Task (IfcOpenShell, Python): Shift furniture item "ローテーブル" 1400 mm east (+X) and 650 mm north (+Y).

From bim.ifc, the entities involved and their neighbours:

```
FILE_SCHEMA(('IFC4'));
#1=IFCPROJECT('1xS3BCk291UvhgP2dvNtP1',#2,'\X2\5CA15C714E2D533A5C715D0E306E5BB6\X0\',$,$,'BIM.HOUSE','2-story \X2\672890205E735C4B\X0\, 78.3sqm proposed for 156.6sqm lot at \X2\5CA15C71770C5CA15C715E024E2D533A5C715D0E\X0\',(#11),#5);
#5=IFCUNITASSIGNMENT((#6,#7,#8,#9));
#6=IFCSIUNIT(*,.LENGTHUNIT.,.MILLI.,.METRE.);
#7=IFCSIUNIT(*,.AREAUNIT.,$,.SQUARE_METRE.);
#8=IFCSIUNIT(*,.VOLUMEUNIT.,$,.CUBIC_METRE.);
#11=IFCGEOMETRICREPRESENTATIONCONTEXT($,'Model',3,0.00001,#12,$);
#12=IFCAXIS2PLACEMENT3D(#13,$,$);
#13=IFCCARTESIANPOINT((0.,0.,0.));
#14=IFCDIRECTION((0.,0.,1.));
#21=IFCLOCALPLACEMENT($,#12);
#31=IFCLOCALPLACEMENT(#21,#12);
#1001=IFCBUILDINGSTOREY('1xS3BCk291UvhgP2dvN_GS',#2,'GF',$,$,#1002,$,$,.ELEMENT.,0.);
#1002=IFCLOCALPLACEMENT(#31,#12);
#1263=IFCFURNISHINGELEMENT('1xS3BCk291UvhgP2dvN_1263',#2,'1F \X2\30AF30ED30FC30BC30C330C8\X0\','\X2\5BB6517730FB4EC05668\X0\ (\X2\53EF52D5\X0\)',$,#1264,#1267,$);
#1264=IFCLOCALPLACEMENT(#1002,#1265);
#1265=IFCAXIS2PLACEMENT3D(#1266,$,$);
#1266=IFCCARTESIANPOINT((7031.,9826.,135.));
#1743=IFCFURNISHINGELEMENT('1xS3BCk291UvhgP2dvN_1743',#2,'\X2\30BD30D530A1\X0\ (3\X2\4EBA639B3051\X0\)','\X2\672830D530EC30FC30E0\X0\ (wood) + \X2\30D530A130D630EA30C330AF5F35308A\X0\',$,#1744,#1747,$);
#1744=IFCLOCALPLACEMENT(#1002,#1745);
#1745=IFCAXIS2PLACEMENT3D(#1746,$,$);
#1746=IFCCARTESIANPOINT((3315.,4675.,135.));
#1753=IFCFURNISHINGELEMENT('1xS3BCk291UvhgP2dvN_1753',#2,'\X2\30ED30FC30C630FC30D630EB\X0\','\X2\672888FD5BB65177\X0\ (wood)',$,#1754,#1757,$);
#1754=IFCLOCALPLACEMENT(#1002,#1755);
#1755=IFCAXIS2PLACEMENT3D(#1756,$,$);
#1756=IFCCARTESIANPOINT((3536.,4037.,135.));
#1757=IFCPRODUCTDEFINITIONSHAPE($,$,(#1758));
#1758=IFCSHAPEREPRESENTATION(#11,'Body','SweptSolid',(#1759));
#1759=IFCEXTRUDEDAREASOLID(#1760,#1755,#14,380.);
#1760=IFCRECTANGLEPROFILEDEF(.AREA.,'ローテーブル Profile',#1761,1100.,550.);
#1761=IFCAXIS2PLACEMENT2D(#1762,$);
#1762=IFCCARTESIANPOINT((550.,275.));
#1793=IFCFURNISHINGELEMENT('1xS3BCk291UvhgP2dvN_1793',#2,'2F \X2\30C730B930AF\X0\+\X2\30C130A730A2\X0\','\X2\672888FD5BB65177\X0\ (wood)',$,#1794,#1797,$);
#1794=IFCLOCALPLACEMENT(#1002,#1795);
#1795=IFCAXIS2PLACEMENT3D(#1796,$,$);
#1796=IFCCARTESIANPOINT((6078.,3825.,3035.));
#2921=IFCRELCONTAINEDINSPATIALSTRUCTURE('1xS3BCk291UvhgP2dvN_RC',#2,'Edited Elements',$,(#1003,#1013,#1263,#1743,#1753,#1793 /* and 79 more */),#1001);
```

```python
import ifcopenshell
import ifcopenshell.api.geometry
import ifcopenshell.util.placement
import ifcopenshell.util.unit

model = ifcopenshell.open("bim.ifc")
unit_scale = ifcopenshell.util.unit.calculate_unit_scale(model)

item = model.by_id(1753)
matrix = ifcopenshell.util.placement.get_local_placement(item.ObjectPlacement)
matrix[0, 3] += 1.4 / unit_scale
matrix[1, 3] += 0.65 / unit_scale
ifcopenshell.api.geometry.edit_object_placement(model, product=item, matrix=matrix, is_si=False)

print(ifcopenshell.util.placement.get_local_placement(item.ObjectPlacement).round(3) + 0.0)

model.write("bim_rev.ifc")
```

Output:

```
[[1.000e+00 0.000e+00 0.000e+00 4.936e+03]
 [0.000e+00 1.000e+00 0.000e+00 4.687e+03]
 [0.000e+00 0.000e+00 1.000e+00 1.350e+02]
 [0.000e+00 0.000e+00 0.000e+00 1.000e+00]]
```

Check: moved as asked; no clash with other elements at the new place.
